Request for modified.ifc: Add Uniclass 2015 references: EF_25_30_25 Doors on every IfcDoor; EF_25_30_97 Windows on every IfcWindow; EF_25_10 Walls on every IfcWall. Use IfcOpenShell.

First a look at what the model holds.

```python
import ifcopenshell

model = ifcopenshell.open("modified.ifc")
print(model.schema)
print("classifications:", [c.Name for c in model.by_type("IfcClassification")])
for ifc_class in ("IfcDoor", "IfcRoof", "IfcStair", "IfcWall", "IfcWindow"):
    print(ifc_class, len(model.by_type(ifc_class)))
```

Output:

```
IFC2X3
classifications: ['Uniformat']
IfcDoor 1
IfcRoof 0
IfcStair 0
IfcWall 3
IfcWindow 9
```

```python
import ifcopenshell
import ifcopenshell.api.classification

model = ifcopenshell.open("modified.ifc")

# IFC2X3 requires Source and Edition and has no link from the project to the system.
system = model.create_entity("IfcClassification", Source="NBS", Edition="2015", Name="Uniclass 2015")

codes = {
    "IfcDoor": ("EF_25_30_25", "Doors"),
    "IfcWindow": ("EF_25_30_97", "Windows"),
    "IfcWall": ("EF_25_10", "Walls"),
}
for ifc_class, (code, name) in codes.items():
    products = model.by_type(ifc_class)
    ifcopenshell.api.classification.add_reference(
        model, products=products, classification=system, identification=code, name=name
    )
    print(code, len(products))

model.write("modified_rev.ifc")
```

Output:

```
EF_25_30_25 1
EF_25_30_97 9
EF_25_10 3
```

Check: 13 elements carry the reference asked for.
